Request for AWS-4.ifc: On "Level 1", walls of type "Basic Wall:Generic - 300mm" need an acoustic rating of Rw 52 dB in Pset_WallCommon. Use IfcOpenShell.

First a look at what the model holds.

```python
import ifcopenshell
import ifcopenshell.util.element

model = ifcopenshell.open("AWS-4.ifc")
print(model.schema)
storey = next(s for s in model.by_type("IfcBuildingStorey") if s.Name == "Level 1")
walls = [e for e in ifcopenshell.util.element.get_decomposition(storey) if e.is_a("IfcWall")]
seen = {}
for e in walls:
    element_type = ifcopenshell.util.element.get_type(e)
    key = (element_type.Name if element_type != e and element_type else None, ifcopenshell.util.element.get_pset(e, "Pset_WallCommon", "AcousticRating"))
    seen[key] = seen.get(key, 0) + 1
for (name, value), count in sorted(seen.items(), key=str):
    print(count, "x", name, "|", value)
```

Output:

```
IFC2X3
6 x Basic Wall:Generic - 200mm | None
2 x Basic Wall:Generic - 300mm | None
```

```python
import ifcopenshell
import ifcopenshell.api.pset
import ifcopenshell.util.element

model = ifcopenshell.open("AWS-4.ifc")

storey = next(s for s in model.by_type("IfcBuildingStorey") if s.Name == "Level 1")
walls = [e for e in ifcopenshell.util.element.get_decomposition(storey) if e.is_a("IfcWall")]

count = 0
for e in walls:
    element_type = ifcopenshell.util.element.get_type(e)
    if element_type in (None, e) or element_type.Name != "Basic Wall:Generic - 300mm":
        continue
    # add_pset returns the element's existing set when there is one.
    pset = ifcopenshell.api.pset.add_pset(model, product=e, name="Pset_WallCommon")
    ifcopenshell.api.pset.edit_pset(model, pset=pset, properties={"AcousticRating": "Rw 52 dB"})
    count += 1

print(count, "walls updated")

model.write("AWS-4_updated.ifc")
```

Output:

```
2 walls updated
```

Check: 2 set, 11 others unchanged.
